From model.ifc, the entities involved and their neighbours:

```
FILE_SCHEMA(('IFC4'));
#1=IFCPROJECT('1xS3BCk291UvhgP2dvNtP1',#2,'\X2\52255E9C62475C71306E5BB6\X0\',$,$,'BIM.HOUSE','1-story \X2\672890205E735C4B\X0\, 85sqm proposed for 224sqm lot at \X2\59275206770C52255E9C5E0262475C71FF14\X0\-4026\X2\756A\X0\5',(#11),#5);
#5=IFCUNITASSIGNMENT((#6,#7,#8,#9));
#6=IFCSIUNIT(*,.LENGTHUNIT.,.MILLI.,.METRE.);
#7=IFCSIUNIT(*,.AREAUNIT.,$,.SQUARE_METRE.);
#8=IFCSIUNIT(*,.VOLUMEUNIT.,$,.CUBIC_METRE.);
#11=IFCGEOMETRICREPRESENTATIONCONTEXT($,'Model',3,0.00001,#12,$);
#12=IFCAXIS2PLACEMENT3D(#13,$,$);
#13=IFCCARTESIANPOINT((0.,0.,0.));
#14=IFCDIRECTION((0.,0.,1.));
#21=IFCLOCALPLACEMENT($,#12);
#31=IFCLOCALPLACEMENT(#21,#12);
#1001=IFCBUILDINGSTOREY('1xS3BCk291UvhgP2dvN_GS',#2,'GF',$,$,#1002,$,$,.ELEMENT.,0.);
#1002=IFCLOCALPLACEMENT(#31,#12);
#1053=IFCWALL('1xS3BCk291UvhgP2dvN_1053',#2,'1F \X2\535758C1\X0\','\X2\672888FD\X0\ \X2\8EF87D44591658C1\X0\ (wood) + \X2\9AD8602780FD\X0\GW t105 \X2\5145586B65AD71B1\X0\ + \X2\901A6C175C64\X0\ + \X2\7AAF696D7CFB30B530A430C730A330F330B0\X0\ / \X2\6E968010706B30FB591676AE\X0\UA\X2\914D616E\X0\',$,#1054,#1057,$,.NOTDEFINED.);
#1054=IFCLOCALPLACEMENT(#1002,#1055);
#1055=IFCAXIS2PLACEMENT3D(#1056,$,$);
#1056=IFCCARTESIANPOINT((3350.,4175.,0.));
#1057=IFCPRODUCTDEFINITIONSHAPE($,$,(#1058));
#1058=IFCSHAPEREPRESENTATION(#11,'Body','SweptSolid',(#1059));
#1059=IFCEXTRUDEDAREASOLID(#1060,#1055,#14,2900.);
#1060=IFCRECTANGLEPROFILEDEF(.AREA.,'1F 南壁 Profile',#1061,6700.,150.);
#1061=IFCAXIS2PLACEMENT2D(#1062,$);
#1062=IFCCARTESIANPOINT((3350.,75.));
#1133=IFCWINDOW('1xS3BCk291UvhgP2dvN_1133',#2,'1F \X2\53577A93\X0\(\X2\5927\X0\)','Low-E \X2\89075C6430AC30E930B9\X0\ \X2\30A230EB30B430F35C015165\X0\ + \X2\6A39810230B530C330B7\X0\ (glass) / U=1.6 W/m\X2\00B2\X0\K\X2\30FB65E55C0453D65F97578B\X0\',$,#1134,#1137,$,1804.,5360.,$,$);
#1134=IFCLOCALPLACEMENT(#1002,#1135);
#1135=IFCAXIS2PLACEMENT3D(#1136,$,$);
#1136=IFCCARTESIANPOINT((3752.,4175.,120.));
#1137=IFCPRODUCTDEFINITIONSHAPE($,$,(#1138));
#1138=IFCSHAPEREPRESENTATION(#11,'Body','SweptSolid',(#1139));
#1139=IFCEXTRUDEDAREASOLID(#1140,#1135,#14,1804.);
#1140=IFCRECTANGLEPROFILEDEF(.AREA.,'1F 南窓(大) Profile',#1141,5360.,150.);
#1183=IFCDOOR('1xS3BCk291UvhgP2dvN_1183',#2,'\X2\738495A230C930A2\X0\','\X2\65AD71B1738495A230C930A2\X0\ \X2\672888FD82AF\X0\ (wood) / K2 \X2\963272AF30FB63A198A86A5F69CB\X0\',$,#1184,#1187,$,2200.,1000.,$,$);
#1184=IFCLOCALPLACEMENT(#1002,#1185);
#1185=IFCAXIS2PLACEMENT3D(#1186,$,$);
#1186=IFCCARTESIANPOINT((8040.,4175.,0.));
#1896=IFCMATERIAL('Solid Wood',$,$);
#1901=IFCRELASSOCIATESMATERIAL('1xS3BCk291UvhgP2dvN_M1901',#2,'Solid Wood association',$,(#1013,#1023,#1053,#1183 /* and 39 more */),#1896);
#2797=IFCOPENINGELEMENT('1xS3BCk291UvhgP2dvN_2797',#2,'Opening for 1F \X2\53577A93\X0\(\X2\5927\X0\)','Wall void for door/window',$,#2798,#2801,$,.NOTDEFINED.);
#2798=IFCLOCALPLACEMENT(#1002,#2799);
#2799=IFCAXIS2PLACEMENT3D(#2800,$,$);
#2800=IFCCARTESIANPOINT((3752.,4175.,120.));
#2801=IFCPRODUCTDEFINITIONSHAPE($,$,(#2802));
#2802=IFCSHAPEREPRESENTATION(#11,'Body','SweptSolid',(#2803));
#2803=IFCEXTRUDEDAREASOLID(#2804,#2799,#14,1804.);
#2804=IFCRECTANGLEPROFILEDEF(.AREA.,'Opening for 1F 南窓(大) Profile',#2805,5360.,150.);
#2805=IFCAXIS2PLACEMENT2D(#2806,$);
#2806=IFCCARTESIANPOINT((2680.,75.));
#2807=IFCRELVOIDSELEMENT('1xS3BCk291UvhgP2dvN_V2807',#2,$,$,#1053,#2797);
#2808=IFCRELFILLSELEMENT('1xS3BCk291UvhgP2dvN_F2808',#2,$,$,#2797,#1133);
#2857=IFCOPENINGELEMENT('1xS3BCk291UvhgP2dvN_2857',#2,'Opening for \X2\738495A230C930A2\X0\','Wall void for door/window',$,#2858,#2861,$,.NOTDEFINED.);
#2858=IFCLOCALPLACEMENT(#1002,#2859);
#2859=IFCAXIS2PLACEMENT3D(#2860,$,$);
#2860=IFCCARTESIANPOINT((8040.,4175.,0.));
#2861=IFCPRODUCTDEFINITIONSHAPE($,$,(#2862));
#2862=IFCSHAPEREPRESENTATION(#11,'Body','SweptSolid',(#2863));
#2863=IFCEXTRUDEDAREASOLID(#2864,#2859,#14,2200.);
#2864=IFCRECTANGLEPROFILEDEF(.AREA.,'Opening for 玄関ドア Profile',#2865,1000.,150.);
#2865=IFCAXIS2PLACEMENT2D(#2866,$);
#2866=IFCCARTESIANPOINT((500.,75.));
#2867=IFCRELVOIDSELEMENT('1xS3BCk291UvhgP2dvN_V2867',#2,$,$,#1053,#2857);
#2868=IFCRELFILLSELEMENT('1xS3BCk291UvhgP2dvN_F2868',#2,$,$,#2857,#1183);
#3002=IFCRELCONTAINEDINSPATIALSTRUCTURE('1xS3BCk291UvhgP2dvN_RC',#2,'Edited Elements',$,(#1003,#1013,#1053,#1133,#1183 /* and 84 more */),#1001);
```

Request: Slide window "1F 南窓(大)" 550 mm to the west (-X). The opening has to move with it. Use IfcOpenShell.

```python
import ifcopenshell
import ifcopenshell.api.geometry
import ifcopenshell.util.placement
import ifcopenshell.util.unit

model = ifcopenshell.open("model.ifc")
unit_scale = ifcopenshell.util.unit.calculate_unit_scale(model)

window = model.by_guid("1xS3BCk291UvhgP2dvN_1133")
opening = window.FillsVoids[0].RelatingOpeningElement
wall = opening.VoidsElements[0].RelatingBuildingElement

wall_matrix = ifcopenshell.util.placement.get_local_placement(wall.ObjectPlacement)
shift = wall_matrix[:3, 0] * -0.55 / unit_scale
before = ifcopenshell.util.placement.get_local_placement(window.ObjectPlacement)[:3, 3].copy()

# The window is not placed relative to its opening, so move both.
for product in (opening, window):
    matrix = ifcopenshell.util.placement.get_local_placement(product.ObjectPlacement)
    matrix[:3, 3] += shift
    ifcopenshell.api.geometry.edit_object_placement(model, product=product, matrix=matrix, is_si=False)

after = ifcopenshell.util.placement.get_local_placement(window.ObjectPlacement)[:3, 3]
print("window moved by", (after - before).round(3) + 0.0)

model.write("model_rev.ifc")
```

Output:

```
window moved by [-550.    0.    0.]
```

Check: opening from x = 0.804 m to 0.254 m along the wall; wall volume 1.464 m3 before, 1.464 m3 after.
